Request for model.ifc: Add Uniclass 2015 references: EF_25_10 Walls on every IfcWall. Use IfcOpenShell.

First a look at what the model holds.

```python
import ifcopenshell

model = ifcopenshell.open("model.ifc")
print(model.schema)
print("classifications:", [c.Name for c in model.by_type("IfcClassification")])
for ifc_class in ("IfcDoor", "IfcRoof", "IfcStair", "IfcWall", "IfcWindow"):
    print(ifc_class, len(model.by_type(ifc_class)))
```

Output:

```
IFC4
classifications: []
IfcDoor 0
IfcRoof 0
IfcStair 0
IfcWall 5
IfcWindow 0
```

```python
import ifcopenshell
import ifcopenshell.api.classification

model = ifcopenshell.open("model.ifc")

system = ifcopenshell.api.classification.add_classification(model, classification="Uniclass 2015")

codes = {
    "IfcWall": ("EF_25_10", "Walls"),
}
for ifc_class, (code, name) in codes.items():
    products = model.by_type(ifc_class)
    ifcopenshell.api.classification.add_reference(
        model, products=products, classification=system, identification=code, name=name
    )
    print(code, len(products))

model.write("model_v2.ifc")
```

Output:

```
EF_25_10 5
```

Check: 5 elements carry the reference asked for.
